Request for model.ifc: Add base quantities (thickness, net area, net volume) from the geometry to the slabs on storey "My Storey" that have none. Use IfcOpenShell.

First a look at what the model holds.

```python
import ifcopenshell
import ifcopenshell.util.element
import ifcopenshell.util.unit

model = ifcopenshell.open("model.ifc")
print(model.schema)
for unit_type in ("LENGTHUNIT", "AREAUNIT", "VOLUMEUNIT"):
    print(unit_type, ifcopenshell.util.unit.calculate_unit_scale(model, unit_type))
storey = next(s for s in model.by_type("IfcBuildingStorey") if s.Name == "My Storey")
slabs = [e for e in ifcopenshell.util.element.get_decomposition(storey) if e.is_a("IfcSlab")]
for e in sorted(slabs, key=lambda e: e.id()):
    print(e.id(), e.is_a(), e.Name, list(ifcopenshell.util.element.get_psets(e, qtos_only=True)), sep=" | ")
```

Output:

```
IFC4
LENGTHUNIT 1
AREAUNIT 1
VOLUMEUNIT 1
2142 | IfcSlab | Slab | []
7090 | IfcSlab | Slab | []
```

```python
import ifcopenshell
import ifcopenshell.api.pset
import ifcopenshell.geom
import ifcopenshell.util.element
import ifcopenshell.util.shape
import ifcopenshell.util.unit

model = ifcopenshell.open("model.ifc")
unit_scale = ifcopenshell.util.unit.calculate_unit_scale(model)
area_scale = ifcopenshell.util.unit.calculate_unit_scale(model, "AREAUNIT")
volume_scale = ifcopenshell.util.unit.calculate_unit_scale(model, "VOLUMEUNIT")
settings = ifcopenshell.geom.settings()

storey = next(s for s in model.by_type("IfcBuildingStorey") if s.Name == "My Storey")
slabs = [e for e in ifcopenshell.util.element.get_decomposition(storey) if e.is_a("IfcSlab")]

for e in sorted(slabs, key=lambda e: e.id()):
    if ifcopenshell.util.element.get_psets(e, qtos_only=True, should_inherit=False):
        continue
    # Geometry comes back in metres, in the element's own axes.
    shape = ifcopenshell.geom.create_shape(settings, e)
    values = {
        "Width": ifcopenshell.util.shape.get_z(shape.geometry) / unit_scale,
        "NetArea": ifcopenshell.util.shape.get_footprint_area(shape.geometry) / area_scale,
        "NetVolume": ifcopenshell.util.shape.get_volume(shape.geometry) / volume_scale,
    }
    qto = ifcopenshell.api.pset.add_qto(model, product=e, name="Qto_SlabBaseQuantities")
    ifcopenshell.api.pset.edit_qto(model, qto=qto, properties=values)
    print(e.id(), {k: round(v, 3) for k, v in values.items()})

model.write("model_v2.ifc")
```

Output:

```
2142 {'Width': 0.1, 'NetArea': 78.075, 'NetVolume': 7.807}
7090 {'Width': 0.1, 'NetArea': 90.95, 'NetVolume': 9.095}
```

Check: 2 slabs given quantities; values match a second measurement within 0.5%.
